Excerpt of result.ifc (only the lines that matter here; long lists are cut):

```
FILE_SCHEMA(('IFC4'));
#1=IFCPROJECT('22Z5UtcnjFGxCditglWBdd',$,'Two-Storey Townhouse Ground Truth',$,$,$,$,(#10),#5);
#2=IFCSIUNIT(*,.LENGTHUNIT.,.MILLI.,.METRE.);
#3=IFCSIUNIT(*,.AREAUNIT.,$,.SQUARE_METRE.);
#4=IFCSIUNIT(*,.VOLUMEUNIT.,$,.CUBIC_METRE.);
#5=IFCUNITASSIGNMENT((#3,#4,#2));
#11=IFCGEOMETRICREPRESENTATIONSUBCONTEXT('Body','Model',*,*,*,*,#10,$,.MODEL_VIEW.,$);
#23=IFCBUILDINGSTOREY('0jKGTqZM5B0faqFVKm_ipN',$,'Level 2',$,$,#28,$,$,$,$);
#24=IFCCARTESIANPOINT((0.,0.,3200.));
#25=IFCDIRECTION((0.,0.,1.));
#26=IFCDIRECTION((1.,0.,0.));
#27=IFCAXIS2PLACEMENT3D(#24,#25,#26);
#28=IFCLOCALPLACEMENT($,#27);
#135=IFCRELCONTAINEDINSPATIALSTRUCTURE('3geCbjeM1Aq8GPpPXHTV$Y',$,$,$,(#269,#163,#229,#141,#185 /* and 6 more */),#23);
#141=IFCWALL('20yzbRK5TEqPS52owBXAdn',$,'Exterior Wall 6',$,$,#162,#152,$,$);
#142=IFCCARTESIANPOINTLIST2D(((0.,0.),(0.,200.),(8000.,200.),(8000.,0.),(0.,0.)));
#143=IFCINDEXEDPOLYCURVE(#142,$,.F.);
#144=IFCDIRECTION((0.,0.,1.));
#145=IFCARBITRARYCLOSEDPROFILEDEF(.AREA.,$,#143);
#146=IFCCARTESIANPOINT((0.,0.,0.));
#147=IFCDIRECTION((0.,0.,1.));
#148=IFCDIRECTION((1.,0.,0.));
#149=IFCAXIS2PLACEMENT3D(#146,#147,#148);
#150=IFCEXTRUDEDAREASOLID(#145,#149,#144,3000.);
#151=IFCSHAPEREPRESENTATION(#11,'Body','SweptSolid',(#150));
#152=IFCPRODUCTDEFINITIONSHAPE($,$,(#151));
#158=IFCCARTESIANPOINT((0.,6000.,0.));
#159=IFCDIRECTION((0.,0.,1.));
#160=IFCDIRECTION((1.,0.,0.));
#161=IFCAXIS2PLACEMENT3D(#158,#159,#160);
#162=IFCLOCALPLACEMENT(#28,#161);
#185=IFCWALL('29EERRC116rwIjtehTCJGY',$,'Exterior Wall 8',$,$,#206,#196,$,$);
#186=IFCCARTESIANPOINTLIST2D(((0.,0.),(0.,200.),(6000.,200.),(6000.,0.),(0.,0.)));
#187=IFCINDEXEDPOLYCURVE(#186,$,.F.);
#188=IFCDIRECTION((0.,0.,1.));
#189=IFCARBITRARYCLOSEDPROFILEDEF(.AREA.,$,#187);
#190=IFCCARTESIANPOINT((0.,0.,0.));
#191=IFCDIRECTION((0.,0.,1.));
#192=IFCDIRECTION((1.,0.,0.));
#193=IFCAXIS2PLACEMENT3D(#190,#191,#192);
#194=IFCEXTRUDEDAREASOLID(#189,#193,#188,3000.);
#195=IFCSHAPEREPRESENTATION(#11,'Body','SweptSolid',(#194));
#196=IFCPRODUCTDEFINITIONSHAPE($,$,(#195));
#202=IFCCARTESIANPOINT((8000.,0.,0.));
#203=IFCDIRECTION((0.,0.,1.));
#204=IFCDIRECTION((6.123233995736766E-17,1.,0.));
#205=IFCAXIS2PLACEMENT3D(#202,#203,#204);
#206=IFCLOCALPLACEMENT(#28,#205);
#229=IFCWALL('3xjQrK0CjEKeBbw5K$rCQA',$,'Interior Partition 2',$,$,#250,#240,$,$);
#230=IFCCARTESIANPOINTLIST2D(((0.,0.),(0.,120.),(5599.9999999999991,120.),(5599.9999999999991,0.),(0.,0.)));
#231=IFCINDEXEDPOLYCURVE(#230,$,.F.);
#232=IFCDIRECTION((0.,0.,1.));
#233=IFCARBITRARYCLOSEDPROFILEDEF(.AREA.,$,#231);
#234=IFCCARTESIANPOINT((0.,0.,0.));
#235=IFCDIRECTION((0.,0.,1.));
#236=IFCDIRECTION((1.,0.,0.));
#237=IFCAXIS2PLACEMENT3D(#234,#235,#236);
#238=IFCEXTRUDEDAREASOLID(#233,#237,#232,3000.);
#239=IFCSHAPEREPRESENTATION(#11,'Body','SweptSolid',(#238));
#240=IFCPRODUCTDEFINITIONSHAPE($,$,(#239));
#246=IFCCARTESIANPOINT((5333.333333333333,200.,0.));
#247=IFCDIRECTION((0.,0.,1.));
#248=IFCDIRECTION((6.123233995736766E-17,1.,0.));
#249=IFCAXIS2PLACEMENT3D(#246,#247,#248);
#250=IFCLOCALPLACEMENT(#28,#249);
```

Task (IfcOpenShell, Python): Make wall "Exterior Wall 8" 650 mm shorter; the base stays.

```python
import ifcopenshell
import ifcopenshell.geom
import ifcopenshell.util.representation
import ifcopenshell.util.shape
import ifcopenshell.util.unit

model = ifcopenshell.open("result.ifc")
unit_scale = ifcopenshell.util.unit.calculate_unit_scale(model)
settings = ifcopenshell.geom.settings()


def volume(element):
    """Net volume in cubic metres, openings subtracted."""
    shape = ifcopenshell.geom.create_shape(settings, element)
    return ifcopenshell.util.shape.get_volume(shape.geometry)


wall = model.by_guid("29EERRC116rwIjtehTCJGY")
before = volume(wall)

body = ifcopenshell.util.representation.get_representation(wall, "Model", "Body")
solid = body.Items[0]
old_height = solid.Depth
solid.Depth -= 0.65 / unit_scale
after = volume(wall)

print(f"height {old_height:g} -> {solid.Depth:g}, volume {before:.3f} -> {after:.3f} m3")

model.write("result_rev.ifc")
```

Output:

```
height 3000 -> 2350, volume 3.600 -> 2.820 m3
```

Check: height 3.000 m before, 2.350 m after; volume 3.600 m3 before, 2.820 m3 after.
